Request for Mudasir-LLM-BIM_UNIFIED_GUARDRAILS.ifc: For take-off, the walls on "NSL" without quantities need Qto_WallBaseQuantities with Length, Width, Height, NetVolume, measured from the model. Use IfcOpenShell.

First a look at what the model holds.

```python
import ifcopenshell
import ifcopenshell.util.element
import ifcopenshell.util.unit

model = ifcopenshell.open("Mudasir-LLM-BIM_UNIFIED_GUARDRAILS.ifc")
print(model.schema)
for unit_type in ("LENGTHUNIT", "AREAUNIT", "VOLUMEUNIT"):
    print(unit_type, ifcopenshell.util.unit.calculate_unit_scale(model, unit_type))
storey = next(s for s in model.by_type("IfcBuildingStorey") if s.Name == "NSL")
walls = [e for e in ifcopenshell.util.element.get_decomposition(storey) if e.is_a("IfcWall")]
for e in sorted(walls, key=lambda e: e.id()):
    print(e.id(), e.is_a(), e.Name, list(ifcopenshell.util.element.get_psets(e, qtos_only=True)), sep=" | ")
```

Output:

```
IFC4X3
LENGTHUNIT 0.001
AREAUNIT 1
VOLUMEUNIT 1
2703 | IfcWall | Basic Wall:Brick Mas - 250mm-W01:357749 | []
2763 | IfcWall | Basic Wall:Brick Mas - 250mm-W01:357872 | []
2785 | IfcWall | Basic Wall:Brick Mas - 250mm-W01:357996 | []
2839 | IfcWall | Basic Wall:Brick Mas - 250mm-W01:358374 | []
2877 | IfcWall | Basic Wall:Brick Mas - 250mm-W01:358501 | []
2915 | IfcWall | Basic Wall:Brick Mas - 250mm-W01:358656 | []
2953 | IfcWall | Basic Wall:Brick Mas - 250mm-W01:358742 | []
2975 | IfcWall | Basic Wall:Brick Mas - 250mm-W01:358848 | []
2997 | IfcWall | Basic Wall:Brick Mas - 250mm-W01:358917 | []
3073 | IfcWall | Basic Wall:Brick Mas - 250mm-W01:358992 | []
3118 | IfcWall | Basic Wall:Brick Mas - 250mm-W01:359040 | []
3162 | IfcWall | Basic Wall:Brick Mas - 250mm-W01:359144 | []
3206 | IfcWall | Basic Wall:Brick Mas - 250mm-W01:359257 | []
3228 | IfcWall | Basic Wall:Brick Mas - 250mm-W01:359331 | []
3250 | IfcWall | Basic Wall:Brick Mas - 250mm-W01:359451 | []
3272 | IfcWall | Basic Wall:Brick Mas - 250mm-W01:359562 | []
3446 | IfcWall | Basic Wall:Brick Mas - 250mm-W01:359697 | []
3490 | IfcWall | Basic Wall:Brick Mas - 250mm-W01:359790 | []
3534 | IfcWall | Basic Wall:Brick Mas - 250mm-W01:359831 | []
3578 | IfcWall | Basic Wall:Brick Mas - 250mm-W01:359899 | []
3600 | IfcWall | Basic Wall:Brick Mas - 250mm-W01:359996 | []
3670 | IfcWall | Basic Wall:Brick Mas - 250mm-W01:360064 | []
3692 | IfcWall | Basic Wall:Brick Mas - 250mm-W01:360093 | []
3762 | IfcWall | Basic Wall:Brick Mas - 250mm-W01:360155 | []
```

```python
import ifcopenshell
import ifcopenshell.api.pset
import ifcopenshell.geom
import ifcopenshell.util.element
import ifcopenshell.util.shape
import ifcopenshell.util.unit

model = ifcopenshell.open("Mudasir-LLM-BIM_UNIFIED_GUARDRAILS.ifc")
unit_scale = ifcopenshell.util.unit.calculate_unit_scale(model)
volume_scale = ifcopenshell.util.unit.calculate_unit_scale(model, "VOLUMEUNIT")
settings = ifcopenshell.geom.settings()

storey = next(s for s in model.by_type("IfcBuildingStorey") if s.Name == "NSL")
walls = [e for e in ifcopenshell.util.element.get_decomposition(storey) if e.is_a("IfcWall")]

for e in sorted(walls, key=lambda e: e.id()):
    if ifcopenshell.util.element.get_psets(e, qtos_only=True, should_inherit=False):
        continue
    # Geometry comes back in metres, in the element's own axes.
    shape = ifcopenshell.geom.create_shape(settings, e)
    values = {
        "Length": ifcopenshell.util.shape.get_x(shape.geometry) / unit_scale,
        "Width": ifcopenshell.util.shape.get_y(shape.geometry) / unit_scale,
        "Height": ifcopenshell.util.shape.get_z(shape.geometry) / unit_scale,
        "NetVolume": ifcopenshell.util.shape.get_volume(shape.geometry) / volume_scale,
    }
    qto = ifcopenshell.api.pset.add_qto(model, product=e, name="Qto_WallBaseQuantities")
    ifcopenshell.api.pset.edit_qto(model, qto=qto, properties=values)
    print(e.id(), {k: round(v, 3) for k, v in values.items()})

model.write("Mudasir-LLM-BIM_UNIFIED_GUARDRAILS_v2.ifc")
```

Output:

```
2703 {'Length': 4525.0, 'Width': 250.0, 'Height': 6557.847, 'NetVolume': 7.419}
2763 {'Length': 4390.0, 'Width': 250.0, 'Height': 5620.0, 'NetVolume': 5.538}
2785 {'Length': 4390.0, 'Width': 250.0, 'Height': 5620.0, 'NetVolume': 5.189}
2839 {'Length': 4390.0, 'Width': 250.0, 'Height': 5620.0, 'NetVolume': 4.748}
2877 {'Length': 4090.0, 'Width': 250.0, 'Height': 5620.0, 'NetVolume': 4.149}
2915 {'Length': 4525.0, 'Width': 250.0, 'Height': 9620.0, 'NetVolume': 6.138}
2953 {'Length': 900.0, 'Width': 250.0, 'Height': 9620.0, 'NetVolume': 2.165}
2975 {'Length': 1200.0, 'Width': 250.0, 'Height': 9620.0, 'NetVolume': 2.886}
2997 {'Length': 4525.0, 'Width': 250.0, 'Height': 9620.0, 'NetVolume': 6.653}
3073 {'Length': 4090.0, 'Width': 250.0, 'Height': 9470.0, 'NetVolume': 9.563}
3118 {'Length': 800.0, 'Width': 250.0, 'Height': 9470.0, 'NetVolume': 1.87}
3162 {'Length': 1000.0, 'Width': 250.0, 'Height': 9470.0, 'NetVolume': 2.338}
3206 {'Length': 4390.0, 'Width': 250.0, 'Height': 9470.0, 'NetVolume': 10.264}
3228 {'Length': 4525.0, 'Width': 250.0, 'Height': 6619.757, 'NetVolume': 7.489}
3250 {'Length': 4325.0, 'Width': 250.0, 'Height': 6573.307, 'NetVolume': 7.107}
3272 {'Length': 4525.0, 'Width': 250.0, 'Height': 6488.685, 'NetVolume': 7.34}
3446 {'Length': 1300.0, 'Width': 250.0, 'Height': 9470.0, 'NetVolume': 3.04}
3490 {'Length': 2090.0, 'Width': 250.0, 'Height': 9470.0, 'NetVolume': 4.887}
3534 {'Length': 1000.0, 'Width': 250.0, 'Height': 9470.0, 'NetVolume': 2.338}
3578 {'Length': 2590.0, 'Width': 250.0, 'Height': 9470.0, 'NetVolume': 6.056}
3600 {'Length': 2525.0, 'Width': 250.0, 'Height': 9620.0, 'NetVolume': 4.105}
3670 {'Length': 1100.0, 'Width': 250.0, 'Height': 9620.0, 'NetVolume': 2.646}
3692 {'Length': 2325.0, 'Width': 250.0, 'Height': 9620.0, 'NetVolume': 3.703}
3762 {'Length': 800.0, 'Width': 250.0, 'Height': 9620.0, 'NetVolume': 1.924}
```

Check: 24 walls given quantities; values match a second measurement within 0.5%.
